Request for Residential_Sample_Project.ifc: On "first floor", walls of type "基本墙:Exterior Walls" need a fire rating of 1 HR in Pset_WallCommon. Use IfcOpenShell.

First a look at what the model holds.

```python
import ifcopenshell
import ifcopenshell.util.element

model = ifcopenshell.open("Residential_Sample_Project.ifc")
print(model.schema)
storey = next(s for s in model.by_type("IfcBuildingStorey") if s.Name == "first floor")
walls = [e for e in ifcopenshell.util.element.get_decomposition(storey) if e.is_a("IfcWall")]
seen = {}
for e in walls:
    element_type = ifcopenshell.util.element.get_type(e)
    key = (element_type.Name if element_type != e and element_type else None, ifcopenshell.util.element.get_pset(e, "Pset_WallCommon", "FireRating"))
    seen[key] = seen.get(key, 0) + 1
for (name, value), count in sorted(seen.items(), key=str):
    print(count, "x", name, "|", value)
```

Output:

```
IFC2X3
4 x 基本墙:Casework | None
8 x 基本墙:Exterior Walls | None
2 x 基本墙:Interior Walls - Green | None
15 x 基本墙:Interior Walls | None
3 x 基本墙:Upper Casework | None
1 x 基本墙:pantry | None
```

```python
import ifcopenshell
import ifcopenshell.api.pset
import ifcopenshell.util.element

model = ifcopenshell.open("Residential_Sample_Project.ifc")

storey = next(s for s in model.by_type("IfcBuildingStorey") if s.Name == "first floor")
walls = [e for e in ifcopenshell.util.element.get_decomposition(storey) if e.is_a("IfcWall")]

count = 0
for e in walls:
    element_type = ifcopenshell.util.element.get_type(e)
    if element_type in (None, e) or element_type.Name != "基本墙:Exterior Walls":
        continue
    # add_pset returns the element's existing set when there is one.
    pset = ifcopenshell.api.pset.add_pset(model, product=e, name="Pset_WallCommon")
    ifcopenshell.api.pset.edit_pset(model, pset=pset, properties={"FireRating": "1 HR"})
    count += 1

print(count, "walls updated")

model.write("Residential_Sample_Project_v2.ifc")
```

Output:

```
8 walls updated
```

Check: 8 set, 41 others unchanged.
